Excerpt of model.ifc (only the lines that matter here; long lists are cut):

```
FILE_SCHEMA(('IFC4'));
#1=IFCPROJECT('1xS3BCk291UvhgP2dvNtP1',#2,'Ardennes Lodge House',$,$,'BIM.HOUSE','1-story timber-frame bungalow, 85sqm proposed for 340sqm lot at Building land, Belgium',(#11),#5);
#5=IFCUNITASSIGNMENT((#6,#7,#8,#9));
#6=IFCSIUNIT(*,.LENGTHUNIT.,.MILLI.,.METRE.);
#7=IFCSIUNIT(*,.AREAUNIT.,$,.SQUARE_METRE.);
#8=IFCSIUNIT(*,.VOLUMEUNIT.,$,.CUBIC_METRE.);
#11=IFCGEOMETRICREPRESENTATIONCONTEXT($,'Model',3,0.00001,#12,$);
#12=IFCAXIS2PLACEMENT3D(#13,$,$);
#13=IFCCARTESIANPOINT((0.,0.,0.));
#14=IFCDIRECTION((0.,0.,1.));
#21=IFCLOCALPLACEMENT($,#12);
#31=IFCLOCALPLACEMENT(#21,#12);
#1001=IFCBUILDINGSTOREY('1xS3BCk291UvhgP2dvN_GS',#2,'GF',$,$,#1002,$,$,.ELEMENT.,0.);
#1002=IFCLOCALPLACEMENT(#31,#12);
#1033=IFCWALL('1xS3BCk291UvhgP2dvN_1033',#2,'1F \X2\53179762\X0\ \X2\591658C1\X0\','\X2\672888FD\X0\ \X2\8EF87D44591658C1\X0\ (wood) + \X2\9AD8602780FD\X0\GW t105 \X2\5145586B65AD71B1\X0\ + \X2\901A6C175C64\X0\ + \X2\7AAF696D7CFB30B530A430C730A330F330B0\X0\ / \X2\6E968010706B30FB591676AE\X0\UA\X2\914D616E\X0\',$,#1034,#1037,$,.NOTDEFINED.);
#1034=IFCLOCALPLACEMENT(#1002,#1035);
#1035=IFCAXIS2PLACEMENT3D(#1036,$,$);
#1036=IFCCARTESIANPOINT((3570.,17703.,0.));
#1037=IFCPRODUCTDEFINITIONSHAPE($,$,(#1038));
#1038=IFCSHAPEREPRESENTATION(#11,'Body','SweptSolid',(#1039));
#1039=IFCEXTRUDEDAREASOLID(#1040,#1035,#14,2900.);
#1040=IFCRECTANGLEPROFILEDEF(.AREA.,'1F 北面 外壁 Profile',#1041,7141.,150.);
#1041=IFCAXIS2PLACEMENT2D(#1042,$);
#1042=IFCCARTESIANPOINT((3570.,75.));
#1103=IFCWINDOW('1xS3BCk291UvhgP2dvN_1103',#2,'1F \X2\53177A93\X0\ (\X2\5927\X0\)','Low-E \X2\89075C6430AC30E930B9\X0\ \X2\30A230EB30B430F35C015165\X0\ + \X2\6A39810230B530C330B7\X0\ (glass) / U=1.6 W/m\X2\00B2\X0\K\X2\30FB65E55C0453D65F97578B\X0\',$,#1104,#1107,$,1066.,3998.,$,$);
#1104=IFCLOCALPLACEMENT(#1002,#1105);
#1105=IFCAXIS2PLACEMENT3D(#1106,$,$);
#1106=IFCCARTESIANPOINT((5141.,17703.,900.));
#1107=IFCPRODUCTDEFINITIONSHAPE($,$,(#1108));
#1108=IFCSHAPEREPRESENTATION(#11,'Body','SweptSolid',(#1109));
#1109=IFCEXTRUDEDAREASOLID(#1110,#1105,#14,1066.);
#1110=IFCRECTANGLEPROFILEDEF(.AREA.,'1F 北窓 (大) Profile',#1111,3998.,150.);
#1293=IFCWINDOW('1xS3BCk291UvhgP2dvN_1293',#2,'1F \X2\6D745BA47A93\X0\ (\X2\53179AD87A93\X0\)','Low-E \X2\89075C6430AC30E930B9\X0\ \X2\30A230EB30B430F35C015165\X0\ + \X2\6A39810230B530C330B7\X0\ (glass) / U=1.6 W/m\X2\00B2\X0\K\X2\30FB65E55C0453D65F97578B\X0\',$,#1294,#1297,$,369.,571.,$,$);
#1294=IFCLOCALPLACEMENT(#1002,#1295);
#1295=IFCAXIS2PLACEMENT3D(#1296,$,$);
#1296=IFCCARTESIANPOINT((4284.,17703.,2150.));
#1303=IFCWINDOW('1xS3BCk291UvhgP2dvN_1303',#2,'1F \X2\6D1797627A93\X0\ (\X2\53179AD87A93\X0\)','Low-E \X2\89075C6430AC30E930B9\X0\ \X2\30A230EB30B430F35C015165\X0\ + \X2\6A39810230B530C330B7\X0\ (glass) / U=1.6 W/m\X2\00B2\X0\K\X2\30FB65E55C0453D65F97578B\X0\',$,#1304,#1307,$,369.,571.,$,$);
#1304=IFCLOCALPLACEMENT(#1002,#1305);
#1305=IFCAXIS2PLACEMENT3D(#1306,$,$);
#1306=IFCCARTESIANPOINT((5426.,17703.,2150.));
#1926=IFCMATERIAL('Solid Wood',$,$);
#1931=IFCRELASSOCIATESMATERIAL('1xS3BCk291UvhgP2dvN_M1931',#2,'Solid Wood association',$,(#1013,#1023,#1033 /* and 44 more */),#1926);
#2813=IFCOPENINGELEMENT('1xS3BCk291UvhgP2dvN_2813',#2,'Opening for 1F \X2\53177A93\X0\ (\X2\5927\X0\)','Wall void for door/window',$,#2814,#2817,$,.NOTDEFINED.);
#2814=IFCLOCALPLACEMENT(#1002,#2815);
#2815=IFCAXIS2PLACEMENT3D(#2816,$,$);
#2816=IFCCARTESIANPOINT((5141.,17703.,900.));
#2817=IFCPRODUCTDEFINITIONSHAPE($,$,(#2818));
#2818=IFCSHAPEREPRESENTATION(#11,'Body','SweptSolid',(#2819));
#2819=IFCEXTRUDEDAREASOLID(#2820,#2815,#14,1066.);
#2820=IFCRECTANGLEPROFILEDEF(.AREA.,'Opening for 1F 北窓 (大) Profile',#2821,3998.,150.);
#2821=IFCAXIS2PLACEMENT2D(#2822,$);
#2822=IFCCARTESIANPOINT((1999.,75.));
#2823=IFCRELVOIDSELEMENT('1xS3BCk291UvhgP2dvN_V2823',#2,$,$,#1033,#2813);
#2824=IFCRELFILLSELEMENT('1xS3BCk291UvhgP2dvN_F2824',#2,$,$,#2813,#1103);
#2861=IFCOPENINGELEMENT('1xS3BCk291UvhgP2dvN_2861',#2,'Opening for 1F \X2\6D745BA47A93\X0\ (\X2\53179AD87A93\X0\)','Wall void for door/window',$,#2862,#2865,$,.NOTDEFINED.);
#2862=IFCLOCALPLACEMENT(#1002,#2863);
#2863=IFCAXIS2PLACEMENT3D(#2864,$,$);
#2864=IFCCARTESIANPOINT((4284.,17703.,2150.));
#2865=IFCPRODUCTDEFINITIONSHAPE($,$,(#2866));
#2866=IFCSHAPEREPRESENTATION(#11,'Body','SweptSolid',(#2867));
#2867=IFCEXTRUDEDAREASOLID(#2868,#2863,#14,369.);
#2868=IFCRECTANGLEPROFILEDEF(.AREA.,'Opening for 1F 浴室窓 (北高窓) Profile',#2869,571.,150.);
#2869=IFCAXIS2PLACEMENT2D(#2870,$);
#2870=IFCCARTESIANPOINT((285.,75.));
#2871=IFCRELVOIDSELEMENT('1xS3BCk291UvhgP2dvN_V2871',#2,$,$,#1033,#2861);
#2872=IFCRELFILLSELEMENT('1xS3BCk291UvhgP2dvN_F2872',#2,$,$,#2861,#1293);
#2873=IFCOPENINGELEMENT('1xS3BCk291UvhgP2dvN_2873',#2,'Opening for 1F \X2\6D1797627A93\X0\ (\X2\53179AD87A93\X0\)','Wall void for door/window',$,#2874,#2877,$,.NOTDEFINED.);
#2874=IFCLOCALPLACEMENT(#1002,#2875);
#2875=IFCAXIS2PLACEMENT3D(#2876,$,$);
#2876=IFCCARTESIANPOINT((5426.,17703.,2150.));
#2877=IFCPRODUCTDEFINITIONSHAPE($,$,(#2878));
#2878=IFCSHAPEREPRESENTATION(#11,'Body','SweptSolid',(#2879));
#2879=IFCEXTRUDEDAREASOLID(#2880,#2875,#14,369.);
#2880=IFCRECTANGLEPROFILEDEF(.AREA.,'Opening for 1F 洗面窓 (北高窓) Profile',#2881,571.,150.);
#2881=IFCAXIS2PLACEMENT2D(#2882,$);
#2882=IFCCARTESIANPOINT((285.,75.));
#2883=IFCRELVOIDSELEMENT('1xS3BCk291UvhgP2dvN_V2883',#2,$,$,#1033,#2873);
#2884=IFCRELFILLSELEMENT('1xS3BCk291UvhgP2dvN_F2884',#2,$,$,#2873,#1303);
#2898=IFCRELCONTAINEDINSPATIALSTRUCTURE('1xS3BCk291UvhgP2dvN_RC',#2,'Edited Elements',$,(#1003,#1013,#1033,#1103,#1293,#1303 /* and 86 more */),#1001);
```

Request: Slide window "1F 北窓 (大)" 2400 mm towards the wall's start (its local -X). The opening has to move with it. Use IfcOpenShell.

```python
import ifcopenshell
import ifcopenshell.api.geometry
import ifcopenshell.util.placement
import ifcopenshell.util.unit

model = ifcopenshell.open("model.ifc")
unit_scale = ifcopenshell.util.unit.calculate_unit_scale(model)

window = model.by_id(1103)
opening = window.FillsVoids[0].RelatingOpeningElement
wall = opening.VoidsElements[0].RelatingBuildingElement

wall_matrix = ifcopenshell.util.placement.get_local_placement(wall.ObjectPlacement)
shift = wall_matrix[:3, 0] * -2.4 / unit_scale
before = ifcopenshell.util.placement.get_local_placement(window.ObjectPlacement)[:3, 3].copy()

# The window is not placed relative to its opening, so move both.
for product in (opening, window):
    matrix = ifcopenshell.util.placement.get_local_placement(product.ObjectPlacement)
    matrix[:3, 3] += shift
    ifcopenshell.api.geometry.edit_object_placement(model, product=product, matrix=matrix, is_si=False)

after = ifcopenshell.util.placement.get_local_placement(window.ObjectPlacement)[:3, 3]
print("window moved by", (after - before).round(3) + 0.0)

model.write("model_rev.ifc")
```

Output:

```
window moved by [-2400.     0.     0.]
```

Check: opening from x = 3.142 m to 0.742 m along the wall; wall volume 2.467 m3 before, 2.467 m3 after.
